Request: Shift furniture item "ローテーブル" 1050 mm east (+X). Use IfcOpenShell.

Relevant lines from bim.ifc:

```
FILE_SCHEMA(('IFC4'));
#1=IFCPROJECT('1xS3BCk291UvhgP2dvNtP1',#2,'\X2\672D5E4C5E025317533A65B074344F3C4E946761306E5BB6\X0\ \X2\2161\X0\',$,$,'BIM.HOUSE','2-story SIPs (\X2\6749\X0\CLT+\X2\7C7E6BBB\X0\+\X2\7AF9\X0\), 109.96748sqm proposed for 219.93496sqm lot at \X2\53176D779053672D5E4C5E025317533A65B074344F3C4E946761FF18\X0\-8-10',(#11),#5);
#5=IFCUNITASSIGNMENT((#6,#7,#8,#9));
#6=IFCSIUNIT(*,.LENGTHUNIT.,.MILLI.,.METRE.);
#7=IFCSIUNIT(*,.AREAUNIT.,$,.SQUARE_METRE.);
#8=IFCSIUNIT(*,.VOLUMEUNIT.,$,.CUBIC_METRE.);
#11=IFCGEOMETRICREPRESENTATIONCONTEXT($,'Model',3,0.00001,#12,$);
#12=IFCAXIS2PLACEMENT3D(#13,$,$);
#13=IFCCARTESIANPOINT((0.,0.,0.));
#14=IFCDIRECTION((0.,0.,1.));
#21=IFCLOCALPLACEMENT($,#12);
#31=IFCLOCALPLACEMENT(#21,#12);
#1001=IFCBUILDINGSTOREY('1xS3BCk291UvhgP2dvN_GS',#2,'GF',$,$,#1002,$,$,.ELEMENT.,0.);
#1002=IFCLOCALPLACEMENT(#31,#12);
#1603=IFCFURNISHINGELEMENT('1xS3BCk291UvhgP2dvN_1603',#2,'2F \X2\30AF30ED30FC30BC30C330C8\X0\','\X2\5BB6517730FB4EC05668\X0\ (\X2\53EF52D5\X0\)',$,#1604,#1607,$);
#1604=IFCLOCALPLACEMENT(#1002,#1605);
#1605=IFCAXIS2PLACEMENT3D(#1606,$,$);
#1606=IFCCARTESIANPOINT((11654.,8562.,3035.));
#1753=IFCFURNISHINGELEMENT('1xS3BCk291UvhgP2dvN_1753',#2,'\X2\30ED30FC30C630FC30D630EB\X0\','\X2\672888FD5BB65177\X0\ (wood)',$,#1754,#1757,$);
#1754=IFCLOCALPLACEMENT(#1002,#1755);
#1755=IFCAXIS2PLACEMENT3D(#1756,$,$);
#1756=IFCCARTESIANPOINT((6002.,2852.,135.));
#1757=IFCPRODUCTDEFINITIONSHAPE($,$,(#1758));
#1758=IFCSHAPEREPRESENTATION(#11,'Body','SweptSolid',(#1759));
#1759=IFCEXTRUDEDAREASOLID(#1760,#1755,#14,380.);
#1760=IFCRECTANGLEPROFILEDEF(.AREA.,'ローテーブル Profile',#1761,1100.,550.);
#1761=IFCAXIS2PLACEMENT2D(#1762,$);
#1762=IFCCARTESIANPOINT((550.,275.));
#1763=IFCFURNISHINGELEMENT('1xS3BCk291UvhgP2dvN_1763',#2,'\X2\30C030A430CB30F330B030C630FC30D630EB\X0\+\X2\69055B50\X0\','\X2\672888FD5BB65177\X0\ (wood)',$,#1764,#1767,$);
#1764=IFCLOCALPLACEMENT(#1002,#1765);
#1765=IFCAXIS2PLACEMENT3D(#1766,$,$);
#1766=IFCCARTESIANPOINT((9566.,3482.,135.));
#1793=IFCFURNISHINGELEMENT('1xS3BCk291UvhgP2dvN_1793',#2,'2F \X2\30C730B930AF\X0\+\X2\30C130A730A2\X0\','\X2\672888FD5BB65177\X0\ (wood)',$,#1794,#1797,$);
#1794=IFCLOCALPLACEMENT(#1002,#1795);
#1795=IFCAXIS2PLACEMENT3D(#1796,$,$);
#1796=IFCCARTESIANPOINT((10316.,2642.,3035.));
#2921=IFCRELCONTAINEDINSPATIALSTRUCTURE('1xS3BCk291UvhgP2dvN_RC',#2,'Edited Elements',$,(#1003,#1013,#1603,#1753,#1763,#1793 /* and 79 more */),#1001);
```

```python
import ifcopenshell
import ifcopenshell.api.geometry
import ifcopenshell.util.placement
import ifcopenshell.util.unit

model = ifcopenshell.open("bim.ifc")
unit_scale = ifcopenshell.util.unit.calculate_unit_scale(model)

item = model.by_guid("1xS3BCk291UvhgP2dvN_1753")
matrix = ifcopenshell.util.placement.get_local_placement(item.ObjectPlacement)
matrix[0, 3] += 1.05 / unit_scale
ifcopenshell.api.geometry.edit_object_placement(model, product=item, matrix=matrix, is_si=False)

print(ifcopenshell.util.placement.get_local_placement(item.ObjectPlacement).round(3) + 0.0)

model.write("bim_v2.ifc")
```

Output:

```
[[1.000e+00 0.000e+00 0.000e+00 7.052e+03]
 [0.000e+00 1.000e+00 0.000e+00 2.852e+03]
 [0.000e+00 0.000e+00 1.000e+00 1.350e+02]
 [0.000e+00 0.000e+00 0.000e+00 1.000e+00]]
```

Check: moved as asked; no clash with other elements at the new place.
